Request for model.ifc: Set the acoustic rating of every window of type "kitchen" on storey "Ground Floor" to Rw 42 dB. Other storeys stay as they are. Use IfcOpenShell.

First a look at what the model holds.

```python
import ifcopenshell
import ifcopenshell.util.element

model = ifcopenshell.open("model.ifc")
print(model.schema)
storey = next(s for s in model.by_type("IfcBuildingStorey") if s.Name == "Ground Floor")
windows = [e for e in ifcopenshell.util.element.get_decomposition(storey) if e.is_a("IfcWindow")]
seen = {}
for e in windows:
    element_type = ifcopenshell.util.element.get_type(e)
    key = (element_type.Name if element_type != e and element_type else None, ifcopenshell.util.element.get_pset(e, "Pset_WindowCommon", "AcousticRating"))
    seen[key] = seen.get(key, 0) + 1
for (name, value), count in sorted(seen.items(), key=str):
    print(count, "x", name, "|", value)
```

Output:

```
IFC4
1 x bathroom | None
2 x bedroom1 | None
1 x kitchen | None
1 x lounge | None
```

```python
import ifcopenshell
import ifcopenshell.api.pset
import ifcopenshell.util.element

model = ifcopenshell.open("model.ifc")

storey = next(s for s in model.by_type("IfcBuildingStorey") if s.Name == "Ground Floor")
windows = [e for e in ifcopenshell.util.element.get_decomposition(storey) if e.is_a("IfcWindow")]

count = 0
for e in windows:
    element_type = ifcopenshell.util.element.get_type(e)
    if element_type in (None, e) or element_type.Name != "kitchen":
        continue
    # add_pset returns the element's existing set when there is one.
    pset = ifcopenshell.api.pset.add_pset(model, product=e, name="Pset_WindowCommon")
    ifcopenshell.api.pset.edit_pset(model, pset=pset, properties={"AcousticRating": "Rw 42 dB"})
    count += 1

print(count, "windows updated")

model.write("model_edited.ifc")
```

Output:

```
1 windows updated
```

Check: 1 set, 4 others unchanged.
